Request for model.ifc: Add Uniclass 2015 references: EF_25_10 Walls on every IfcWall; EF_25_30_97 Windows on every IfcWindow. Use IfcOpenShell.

First a look at what the model holds.

```python
import ifcopenshell

model = ifcopenshell.open("model.ifc")
print(model.schema)
print("classifications:", [c.Name for c in model.by_type("IfcClassification")])
for ifc_class in ("IfcDoor", "IfcRoof", "IfcStair", "IfcWall", "IfcWindow"):
    print(ifc_class, len(model.by_type(ifc_class)))
```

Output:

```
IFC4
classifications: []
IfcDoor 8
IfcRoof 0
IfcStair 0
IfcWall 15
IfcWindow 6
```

```python
import ifcopenshell
import ifcopenshell.api.classification

model = ifcopenshell.open("model.ifc")

system = ifcopenshell.api.classification.add_classification(model, classification="Uniclass 2015")

codes = {
    "IfcWall": ("EF_25_10", "Walls"),
    "IfcWindow": ("EF_25_30_97", "Windows"),
}
for ifc_class, (code, name) in codes.items():
    products = model.by_type(ifc_class)
    ifcopenshell.api.classification.add_reference(
        model, products=products, classification=system, identification=code, name=name
    )
    print(code, len(products))

model.write("model-out.ifc")
```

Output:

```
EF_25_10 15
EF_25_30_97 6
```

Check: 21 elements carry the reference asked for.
